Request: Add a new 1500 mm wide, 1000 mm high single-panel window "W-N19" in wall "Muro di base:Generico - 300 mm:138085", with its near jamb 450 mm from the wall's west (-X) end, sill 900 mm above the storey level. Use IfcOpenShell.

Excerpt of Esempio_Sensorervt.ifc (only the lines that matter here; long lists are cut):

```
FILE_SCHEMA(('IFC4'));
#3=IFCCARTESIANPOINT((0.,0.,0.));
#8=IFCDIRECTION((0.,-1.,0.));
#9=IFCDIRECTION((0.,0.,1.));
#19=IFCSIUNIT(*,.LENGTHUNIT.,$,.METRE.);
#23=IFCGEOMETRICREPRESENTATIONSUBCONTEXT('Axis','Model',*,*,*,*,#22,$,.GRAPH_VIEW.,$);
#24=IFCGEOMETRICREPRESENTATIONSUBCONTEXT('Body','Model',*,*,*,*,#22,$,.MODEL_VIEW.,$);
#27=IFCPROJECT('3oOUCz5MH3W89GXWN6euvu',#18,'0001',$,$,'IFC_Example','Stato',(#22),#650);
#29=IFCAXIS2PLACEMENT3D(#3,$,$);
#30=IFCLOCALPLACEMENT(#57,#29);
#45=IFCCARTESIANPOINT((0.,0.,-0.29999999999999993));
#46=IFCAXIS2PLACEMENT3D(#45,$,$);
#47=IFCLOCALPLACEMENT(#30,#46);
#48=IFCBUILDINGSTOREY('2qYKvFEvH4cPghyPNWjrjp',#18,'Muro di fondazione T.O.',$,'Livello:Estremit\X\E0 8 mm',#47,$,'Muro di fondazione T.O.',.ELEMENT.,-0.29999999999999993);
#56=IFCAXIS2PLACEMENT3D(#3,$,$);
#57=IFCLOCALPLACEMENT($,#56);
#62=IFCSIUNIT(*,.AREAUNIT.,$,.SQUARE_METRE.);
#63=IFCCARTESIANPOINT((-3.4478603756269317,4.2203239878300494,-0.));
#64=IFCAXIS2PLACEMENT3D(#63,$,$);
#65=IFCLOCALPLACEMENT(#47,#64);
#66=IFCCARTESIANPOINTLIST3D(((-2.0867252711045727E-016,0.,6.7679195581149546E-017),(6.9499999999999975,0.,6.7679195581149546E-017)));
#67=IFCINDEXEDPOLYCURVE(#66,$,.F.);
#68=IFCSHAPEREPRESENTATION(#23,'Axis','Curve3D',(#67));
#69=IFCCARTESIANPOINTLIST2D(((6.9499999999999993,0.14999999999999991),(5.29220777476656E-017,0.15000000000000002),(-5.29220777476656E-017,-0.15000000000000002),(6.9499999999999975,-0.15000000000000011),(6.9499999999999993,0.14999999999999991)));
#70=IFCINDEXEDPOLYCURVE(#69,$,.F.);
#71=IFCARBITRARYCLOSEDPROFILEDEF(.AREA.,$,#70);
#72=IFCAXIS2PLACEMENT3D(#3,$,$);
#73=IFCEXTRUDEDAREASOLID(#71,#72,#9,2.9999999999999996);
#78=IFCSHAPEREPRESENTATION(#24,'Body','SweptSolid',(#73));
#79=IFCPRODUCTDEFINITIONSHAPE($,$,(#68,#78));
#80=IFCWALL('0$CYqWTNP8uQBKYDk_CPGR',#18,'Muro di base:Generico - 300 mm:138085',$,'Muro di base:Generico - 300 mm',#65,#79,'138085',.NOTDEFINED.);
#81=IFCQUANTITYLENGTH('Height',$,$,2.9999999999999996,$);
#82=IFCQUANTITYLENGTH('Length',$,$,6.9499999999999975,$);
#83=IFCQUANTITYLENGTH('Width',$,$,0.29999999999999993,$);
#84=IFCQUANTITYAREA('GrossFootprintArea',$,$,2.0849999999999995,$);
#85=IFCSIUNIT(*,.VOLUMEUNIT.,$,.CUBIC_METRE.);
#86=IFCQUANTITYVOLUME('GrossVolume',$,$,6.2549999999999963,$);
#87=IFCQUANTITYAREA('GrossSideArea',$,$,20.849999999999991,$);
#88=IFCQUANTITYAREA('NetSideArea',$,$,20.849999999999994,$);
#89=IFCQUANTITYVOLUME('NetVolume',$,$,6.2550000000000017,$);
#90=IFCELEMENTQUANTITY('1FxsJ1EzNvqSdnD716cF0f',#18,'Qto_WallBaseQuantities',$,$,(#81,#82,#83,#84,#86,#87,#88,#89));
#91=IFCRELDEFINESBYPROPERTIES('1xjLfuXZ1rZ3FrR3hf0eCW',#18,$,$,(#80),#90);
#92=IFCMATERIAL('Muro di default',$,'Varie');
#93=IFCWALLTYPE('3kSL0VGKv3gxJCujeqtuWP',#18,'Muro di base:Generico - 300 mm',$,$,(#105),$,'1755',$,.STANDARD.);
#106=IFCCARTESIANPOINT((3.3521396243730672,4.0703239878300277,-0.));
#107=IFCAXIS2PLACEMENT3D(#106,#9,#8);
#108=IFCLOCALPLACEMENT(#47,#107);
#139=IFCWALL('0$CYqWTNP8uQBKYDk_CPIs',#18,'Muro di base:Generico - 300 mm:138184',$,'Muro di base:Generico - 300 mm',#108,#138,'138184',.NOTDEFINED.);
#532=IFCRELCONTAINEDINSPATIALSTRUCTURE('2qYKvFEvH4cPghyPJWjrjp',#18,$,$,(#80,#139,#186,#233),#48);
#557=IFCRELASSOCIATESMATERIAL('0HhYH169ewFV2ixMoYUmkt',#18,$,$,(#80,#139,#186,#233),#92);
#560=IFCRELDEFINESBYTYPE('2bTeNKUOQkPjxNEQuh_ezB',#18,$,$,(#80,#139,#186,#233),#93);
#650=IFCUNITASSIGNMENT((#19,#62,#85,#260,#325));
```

```python
import numpy as np
import ifcopenshell
import ifcopenshell.api.feature
import ifcopenshell.api.geometry
import ifcopenshell.api.pset
import ifcopenshell.api.root
import ifcopenshell.api.spatial
import ifcopenshell.geom
import ifcopenshell.util.element
import ifcopenshell.util.placement
import ifcopenshell.util.representation
import ifcopenshell.util.shape
import ifcopenshell.util.unit

model = ifcopenshell.open("Esempio_Sensorervt.ifc")
unit_scale = ifcopenshell.util.unit.calculate_unit_scale(model)
area_scale = ifcopenshell.util.unit.calculate_unit_scale(model, "AREAUNIT")
volume_scale = ifcopenshell.util.unit.calculate_unit_scale(model, "VOLUMEUNIT")
settings = ifcopenshell.geom.settings()


def volume(element):
    """Net volume in cubic metres, openings subtracted."""
    shape = ifcopenshell.geom.create_shape(settings, element)
    return ifcopenshell.util.shape.get_volume(shape.geometry)


wall = model.by_guid("0$CYqWTNP8uQBKYDk_CPGR")
storey = ifcopenshell.util.element.get_container(wall, ifc_class="IfcBuildingStorey")
context = ifcopenshell.util.representation.get_context(model, "Model", "Body", "MODEL_VIEW")
before = volume(wall)

width, height, from_end, sill = 1.5, 1, 0.45, 0.9  # metres

# The wall runs along its own X axis, and the end named is its -X end.
wall_shape = ifcopenshell.geom.create_shape(settings, wall)
x, y, z = ifcopenshell.util.shape.get_vertices(wall_shape.geometry).T
start = x.min() + from_end
face, thickness = float(y.min()), float(y.max() - y.min())
wall_matrix = ifcopenshell.util.placement.get_local_placement(wall.ObjectPlacement)
level = ifcopenshell.util.placement.get_local_placement(storey.ObjectPlacement)[2, 3]


def in_wall(x, y):
    """Placement at x, y metres in the wall's axes, at sill height."""
    matrix = wall_matrix.copy()
    matrix[:, 3] = wall_matrix @ np.array([x / unit_scale, y / unit_scale, 0.0, 1.0])
    matrix[2, 3] = level + sill / unit_scale
    return matrix


# Opening: a box that overshoots both wall faces by 50 mm.
opening = ifcopenshell.api.root.create_entity(model, ifc_class="IfcOpeningElement", predefined_type="OPENING")
box = ifcopenshell.api.geometry.add_wall_representation(
    model, context=context, length=width, height=height, thickness=thickness + 0.1
)
ifcopenshell.api.geometry.assign_representation(model, product=opening, representation=box)
ifcopenshell.api.geometry.edit_object_placement(model, product=opening, matrix=in_wall(start, face - 0.05), is_si=False)
ifcopenshell.api.feature.add_feature(model, feature=opening, element=wall)

window = ifcopenshell.api.root.create_entity(model, ifc_class="IfcWindow", name="W-N19", predefined_type="WINDOW")
window.OverallWidth, window.OverallHeight = width / unit_scale, height / unit_scale
window.PartitioningType = "SINGLE_PANEL"
body = ifcopenshell.api.geometry.add_window_representation(
    model,
    context=context,
    overall_width=window.OverallWidth,
    overall_height=window.OverallHeight,
    partition_type="SINGLE_PANEL",
)
ifcopenshell.api.geometry.assign_representation(model, product=window, representation=body)
ifcopenshell.api.spatial.assign_container(model, products=[window], relating_structure=storey)
ifcopenshell.api.feature.add_filling(model, opening=opening, element=window)

# Centre the window in the wall's thickness.
ifcopenshell.api.geometry.edit_object_placement(model, product=window, matrix=in_wall(start, face), is_si=False)
window_shape = ifcopenshell.geom.create_shape(settings, window)
depth = ifcopenshell.util.shape.get_vertices(window_shape.geometry)[:, 1]
offset = face + thickness / 2 - (depth.min() + depth.max()) / 2
ifcopenshell.api.geometry.edit_object_placement(model, product=window, matrix=in_wall(start, offset), is_si=False)

after = volume(wall)

# Update the wall's stored quantities.
qto = model.by_id(ifcopenshell.util.element.get_pset(wall, "Qto_WallBaseQuantities", should_inherit=False)["id"])
ifcopenshell.api.pset.edit_qto(model, qto=qto, properties={
    "NetSideArea": after / thickness / area_scale,
    "NetVolume": after / volume_scale,
})

print(f"wall volume {before:.3f} -> {after:.3f} m3")

model.write("Esempio_Sensorervt-out.ifc")
```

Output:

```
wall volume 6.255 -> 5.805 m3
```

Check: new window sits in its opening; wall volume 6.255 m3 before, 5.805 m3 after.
